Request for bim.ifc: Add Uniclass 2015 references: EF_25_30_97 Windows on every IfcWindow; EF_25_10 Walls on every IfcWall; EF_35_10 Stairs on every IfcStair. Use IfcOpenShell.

First a look at what the model holds.

```python
import ifcopenshell

model = ifcopenshell.open("bim.ifc")
print(model.schema)
print("classifications:", [c.Name for c in model.by_type("IfcClassification")])
for ifc_class in ("IfcDoor", "IfcRoof", "IfcStair", "IfcWall", "IfcWindow"):
    print(ifc_class, len(model.by_type(ifc_class)))
```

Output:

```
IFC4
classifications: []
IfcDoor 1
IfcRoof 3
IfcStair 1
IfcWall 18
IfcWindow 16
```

```python
import ifcopenshell
import ifcopenshell.api.classification

model = ifcopenshell.open("bim.ifc")

system = ifcopenshell.api.classification.add_classification(model, classification="Uniclass 2015")

codes = {
    "IfcWindow": ("EF_25_30_97", "Windows"),
    "IfcWall": ("EF_25_10", "Walls"),
    "IfcStair": ("EF_35_10", "Stairs"),
}
for ifc_class, (code, name) in codes.items():
    products = model.by_type(ifc_class)
    ifcopenshell.api.classification.add_reference(
        model, products=products, classification=system, identification=code, name=name
    )
    print(code, len(products))

model.write("bim-out.ifc")
```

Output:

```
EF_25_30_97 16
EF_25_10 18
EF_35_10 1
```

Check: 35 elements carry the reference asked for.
